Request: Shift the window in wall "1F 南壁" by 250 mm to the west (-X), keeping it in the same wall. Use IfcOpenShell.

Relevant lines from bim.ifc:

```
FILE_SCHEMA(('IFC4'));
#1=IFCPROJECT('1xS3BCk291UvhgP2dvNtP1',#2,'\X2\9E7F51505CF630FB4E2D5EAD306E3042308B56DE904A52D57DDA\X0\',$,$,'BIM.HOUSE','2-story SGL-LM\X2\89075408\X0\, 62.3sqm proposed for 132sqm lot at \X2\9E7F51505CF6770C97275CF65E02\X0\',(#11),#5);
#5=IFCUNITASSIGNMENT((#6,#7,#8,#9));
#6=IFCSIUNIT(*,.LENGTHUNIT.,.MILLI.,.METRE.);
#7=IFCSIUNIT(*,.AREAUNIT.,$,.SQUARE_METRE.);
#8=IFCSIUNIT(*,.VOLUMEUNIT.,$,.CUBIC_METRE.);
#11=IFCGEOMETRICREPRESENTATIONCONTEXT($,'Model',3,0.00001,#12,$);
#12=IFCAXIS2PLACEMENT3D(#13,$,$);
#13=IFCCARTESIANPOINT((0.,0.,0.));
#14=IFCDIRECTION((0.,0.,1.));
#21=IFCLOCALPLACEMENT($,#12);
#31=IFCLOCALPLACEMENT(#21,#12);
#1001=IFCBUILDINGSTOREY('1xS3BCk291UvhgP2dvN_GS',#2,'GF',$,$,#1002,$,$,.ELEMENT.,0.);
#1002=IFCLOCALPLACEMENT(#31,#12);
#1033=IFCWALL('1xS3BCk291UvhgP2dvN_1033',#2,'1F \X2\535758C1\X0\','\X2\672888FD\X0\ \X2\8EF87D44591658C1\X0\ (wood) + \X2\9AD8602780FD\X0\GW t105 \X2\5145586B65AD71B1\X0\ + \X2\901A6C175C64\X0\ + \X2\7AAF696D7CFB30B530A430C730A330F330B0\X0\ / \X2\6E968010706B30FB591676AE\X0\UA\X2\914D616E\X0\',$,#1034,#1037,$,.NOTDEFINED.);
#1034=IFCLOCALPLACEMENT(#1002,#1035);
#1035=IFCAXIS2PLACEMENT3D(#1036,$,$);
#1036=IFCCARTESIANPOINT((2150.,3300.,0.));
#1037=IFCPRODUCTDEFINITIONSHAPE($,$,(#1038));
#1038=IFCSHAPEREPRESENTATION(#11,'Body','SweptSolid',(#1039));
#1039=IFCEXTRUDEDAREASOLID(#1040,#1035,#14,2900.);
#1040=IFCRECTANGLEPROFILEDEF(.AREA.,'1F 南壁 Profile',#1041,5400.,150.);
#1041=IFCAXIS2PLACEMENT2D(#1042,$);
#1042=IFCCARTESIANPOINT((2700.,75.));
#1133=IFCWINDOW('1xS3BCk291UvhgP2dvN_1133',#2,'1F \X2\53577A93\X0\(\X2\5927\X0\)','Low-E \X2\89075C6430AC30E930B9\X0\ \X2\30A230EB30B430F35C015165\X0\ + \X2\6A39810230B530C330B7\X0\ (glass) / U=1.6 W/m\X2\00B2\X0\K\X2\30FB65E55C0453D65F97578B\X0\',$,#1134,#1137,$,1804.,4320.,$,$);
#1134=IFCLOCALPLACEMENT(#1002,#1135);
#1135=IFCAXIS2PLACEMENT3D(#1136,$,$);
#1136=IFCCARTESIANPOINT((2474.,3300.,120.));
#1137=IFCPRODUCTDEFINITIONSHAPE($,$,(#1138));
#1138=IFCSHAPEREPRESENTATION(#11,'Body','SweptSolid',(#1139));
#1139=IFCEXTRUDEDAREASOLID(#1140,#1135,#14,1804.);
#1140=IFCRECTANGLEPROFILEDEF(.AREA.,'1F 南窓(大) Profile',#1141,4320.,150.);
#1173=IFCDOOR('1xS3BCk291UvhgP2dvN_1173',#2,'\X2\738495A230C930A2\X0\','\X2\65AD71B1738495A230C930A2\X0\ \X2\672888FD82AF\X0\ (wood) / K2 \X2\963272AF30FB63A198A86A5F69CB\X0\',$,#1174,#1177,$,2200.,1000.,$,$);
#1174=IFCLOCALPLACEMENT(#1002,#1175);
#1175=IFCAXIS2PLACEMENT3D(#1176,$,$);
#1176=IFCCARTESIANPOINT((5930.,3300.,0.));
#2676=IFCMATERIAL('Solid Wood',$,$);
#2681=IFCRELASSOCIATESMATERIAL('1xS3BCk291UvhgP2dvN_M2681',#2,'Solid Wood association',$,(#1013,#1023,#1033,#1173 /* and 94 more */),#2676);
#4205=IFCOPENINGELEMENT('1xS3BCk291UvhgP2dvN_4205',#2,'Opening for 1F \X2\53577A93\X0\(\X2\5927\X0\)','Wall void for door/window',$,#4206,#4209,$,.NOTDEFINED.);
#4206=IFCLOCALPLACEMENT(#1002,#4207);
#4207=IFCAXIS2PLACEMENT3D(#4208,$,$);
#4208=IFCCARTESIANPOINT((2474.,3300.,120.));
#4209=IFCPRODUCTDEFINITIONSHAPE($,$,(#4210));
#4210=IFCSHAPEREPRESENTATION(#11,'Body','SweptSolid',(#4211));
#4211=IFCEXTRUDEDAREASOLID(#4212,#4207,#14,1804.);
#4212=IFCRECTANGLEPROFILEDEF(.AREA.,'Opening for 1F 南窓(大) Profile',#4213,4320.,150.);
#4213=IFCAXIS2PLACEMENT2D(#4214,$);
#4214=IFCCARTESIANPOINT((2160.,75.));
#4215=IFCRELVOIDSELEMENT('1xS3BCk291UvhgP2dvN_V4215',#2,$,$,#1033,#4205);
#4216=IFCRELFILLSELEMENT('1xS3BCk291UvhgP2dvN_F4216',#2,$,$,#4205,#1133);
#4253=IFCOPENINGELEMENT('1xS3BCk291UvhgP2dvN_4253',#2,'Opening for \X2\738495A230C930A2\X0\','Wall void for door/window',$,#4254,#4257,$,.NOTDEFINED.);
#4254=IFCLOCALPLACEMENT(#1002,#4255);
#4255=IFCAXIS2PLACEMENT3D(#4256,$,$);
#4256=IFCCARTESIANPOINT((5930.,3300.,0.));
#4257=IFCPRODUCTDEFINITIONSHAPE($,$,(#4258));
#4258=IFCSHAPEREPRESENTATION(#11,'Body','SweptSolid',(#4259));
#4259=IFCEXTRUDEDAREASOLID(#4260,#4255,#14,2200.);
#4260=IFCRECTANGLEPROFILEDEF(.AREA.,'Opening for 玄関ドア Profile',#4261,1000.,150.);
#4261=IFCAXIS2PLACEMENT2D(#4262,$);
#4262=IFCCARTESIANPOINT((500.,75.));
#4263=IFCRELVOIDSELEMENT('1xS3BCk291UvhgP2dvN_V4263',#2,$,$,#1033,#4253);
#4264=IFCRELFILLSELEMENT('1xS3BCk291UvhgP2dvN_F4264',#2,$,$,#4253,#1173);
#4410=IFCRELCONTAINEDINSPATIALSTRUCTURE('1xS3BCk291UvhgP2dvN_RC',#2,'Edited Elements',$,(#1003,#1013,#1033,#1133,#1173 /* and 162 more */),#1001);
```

```python
import ifcopenshell
import ifcopenshell.api.geometry
import ifcopenshell.util.placement
import ifcopenshell.util.unit

model = ifcopenshell.open("bim.ifc")
unit_scale = ifcopenshell.util.unit.calculate_unit_scale(model)

window = model.by_guid("1xS3BCk291UvhgP2dvN_1133")
opening = window.FillsVoids[0].RelatingOpeningElement
wall = opening.VoidsElements[0].RelatingBuildingElement

wall_matrix = ifcopenshell.util.placement.get_local_placement(wall.ObjectPlacement)
shift = wall_matrix[:3, 0] * -0.25 / unit_scale
before = ifcopenshell.util.placement.get_local_placement(window.ObjectPlacement)[:3, 3].copy()

# The window is not placed relative to its opening, so move both.
for product in (opening, window):
    matrix = ifcopenshell.util.placement.get_local_placement(product.ObjectPlacement)
    matrix[:3, 3] += shift
    ifcopenshell.api.geometry.edit_object_placement(model, product=product, matrix=matrix, is_si=False)

after = ifcopenshell.util.placement.get_local_placement(window.ObjectPlacement)[:3, 3]
print("window moved by", (after - before).round(3) + 0.0)

model.write("bim-out.ifc")
```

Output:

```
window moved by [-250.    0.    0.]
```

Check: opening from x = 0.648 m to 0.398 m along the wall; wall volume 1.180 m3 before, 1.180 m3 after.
